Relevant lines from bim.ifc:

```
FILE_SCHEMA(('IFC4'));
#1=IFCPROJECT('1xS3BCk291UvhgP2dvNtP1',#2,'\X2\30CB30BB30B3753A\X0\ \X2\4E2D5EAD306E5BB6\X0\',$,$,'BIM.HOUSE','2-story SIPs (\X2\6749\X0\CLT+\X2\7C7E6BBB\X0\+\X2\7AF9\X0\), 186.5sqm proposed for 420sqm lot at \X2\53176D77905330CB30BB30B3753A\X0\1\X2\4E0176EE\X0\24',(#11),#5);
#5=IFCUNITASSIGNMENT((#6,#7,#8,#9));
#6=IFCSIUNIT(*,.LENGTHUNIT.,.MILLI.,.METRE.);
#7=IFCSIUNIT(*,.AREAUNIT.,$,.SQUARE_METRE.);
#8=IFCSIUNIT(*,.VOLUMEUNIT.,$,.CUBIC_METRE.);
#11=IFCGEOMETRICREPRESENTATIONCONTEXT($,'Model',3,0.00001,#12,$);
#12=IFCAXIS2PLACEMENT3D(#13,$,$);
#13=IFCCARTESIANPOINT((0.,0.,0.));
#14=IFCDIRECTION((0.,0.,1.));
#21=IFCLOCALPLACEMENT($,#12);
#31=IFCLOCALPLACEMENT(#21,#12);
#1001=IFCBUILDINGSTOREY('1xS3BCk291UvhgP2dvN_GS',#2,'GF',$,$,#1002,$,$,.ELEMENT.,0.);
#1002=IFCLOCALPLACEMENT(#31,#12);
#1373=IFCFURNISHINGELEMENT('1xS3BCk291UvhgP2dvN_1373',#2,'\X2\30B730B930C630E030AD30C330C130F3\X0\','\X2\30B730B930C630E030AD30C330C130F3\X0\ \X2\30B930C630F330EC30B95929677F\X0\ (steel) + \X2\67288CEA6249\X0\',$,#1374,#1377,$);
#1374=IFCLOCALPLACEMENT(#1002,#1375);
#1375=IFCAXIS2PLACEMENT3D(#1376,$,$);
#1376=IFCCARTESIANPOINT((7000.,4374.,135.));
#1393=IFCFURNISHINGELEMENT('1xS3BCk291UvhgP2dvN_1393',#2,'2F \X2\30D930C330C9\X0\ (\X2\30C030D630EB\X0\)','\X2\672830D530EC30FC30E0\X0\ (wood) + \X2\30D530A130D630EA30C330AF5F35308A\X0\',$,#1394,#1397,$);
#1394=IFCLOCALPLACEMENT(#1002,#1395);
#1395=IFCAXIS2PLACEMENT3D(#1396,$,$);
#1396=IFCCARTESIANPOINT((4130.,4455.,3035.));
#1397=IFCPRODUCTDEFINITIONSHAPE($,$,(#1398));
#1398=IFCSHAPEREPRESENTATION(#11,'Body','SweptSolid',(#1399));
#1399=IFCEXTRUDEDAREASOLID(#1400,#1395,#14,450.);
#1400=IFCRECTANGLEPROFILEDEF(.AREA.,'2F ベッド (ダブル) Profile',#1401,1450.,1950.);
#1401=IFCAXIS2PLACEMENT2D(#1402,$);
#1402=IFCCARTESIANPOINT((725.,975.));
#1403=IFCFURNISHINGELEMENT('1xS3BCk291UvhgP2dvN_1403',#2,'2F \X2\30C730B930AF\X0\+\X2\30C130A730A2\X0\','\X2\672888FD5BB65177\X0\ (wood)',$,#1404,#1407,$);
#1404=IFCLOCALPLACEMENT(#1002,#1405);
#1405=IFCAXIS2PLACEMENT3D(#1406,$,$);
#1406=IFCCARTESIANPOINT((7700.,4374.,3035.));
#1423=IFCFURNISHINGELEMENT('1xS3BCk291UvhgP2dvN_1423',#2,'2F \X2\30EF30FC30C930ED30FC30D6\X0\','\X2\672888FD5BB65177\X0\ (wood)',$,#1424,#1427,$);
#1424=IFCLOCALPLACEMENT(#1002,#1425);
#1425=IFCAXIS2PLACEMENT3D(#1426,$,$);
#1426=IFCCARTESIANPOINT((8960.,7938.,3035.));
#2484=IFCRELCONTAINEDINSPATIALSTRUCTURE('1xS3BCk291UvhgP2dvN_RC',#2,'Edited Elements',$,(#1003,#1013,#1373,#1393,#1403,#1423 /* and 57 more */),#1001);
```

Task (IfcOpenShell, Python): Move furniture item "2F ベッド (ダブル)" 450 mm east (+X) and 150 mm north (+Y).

```python
import ifcopenshell
import ifcopenshell.api.geometry
import ifcopenshell.util.placement
import ifcopenshell.util.unit

model = ifcopenshell.open("bim.ifc")
unit_scale = ifcopenshell.util.unit.calculate_unit_scale(model)

item = model.by_id(1393)
matrix = ifcopenshell.util.placement.get_local_placement(item.ObjectPlacement)
matrix[0, 3] += 0.45 / unit_scale
matrix[1, 3] += 0.15 / unit_scale
ifcopenshell.api.geometry.edit_object_placement(model, product=item, matrix=matrix, is_si=False)

print(ifcopenshell.util.placement.get_local_placement(item.ObjectPlacement).round(3) + 0.0)

model.write("bim_updated.ifc")
```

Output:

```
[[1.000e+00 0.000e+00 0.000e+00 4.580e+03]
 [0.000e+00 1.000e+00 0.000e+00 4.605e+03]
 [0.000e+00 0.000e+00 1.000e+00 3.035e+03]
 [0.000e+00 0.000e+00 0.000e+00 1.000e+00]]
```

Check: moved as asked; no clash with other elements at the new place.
